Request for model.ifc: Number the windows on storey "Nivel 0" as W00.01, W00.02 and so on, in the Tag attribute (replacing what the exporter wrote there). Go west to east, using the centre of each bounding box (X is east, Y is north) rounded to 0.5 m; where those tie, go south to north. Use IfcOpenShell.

First a look at what the model holds.

```python
import ifcopenshell
import ifcopenshell.util.element
import ifcopenshell.util.placement

model = ifcopenshell.open("model.ifc")
print(model.schema)
storey = next(s for s in model.by_type("IfcBuildingStorey") if s.Name == "Nivel 0")
windows = [e for e in ifcopenshell.util.element.get_decomposition(storey) if e.is_a("IfcWindow")]
for e in sorted(windows, key=lambda e: e.id()):
    origin = ifcopenshell.util.placement.get_local_placement(e.ObjectPlacement)[:3, 3]
    print(e.id(), e.Tag, e.Name, origin.round(2) + 0.0, sep=" | ")
```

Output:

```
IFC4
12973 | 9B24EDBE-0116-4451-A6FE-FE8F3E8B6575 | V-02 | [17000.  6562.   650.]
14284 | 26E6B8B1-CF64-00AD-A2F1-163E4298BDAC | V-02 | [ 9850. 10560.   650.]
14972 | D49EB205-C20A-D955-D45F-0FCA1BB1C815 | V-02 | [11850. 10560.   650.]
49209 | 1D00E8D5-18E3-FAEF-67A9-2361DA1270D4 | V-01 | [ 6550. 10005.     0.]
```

```python
import ifcopenshell
import ifcopenshell.geom
import ifcopenshell.util.element
import ifcopenshell.util.shape

model = ifcopenshell.open("model.ifc")
settings = ifcopenshell.geom.settings()
settings.set("use-world-coords", True)


def centre(element):
    shape = ifcopenshell.geom.create_shape(settings, element)
    return ifcopenshell.util.shape.get_bbox_centroid(shape.geometry)


storey = next(s for s in model.by_type("IfcBuildingStorey") if s.Name == "Nivel 0")
windows = [e for e in ifcopenshell.util.element.get_decomposition(storey) if e.is_a("IfcWindow")]

# Insertion points can sit at a corner or the storey origin, so sort by the geometry (in metres).
centres = {e: centre(e) for e in windows}
windows.sort(key=lambda e: (round(centres[e][0] / 0.5), centres[e][1]))

for i, e in enumerate(windows, start=1):
    number = f"W00.{i:02d}"
    e.Tag = number
    print(e.id(), number)

model.write("model-out.ifc")
```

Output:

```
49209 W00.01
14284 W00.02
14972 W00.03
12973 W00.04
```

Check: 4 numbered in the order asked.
